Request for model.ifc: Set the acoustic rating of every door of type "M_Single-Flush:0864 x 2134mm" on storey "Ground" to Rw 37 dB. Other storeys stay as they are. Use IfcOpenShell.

First a look at what the model holds.

```python
import ifcopenshell
import ifcopenshell.util.element

model = ifcopenshell.open("model.ifc")
print(model.schema)
storey = next(s for s in model.by_type("IfcBuildingStorey") if s.Name == "Ground")
doors = [e for e in ifcopenshell.util.element.get_decomposition(storey) if e.is_a("IfcDoor")]
seen = {}
for e in doors:
    element_type = ifcopenshell.util.element.get_type(e)
    key = (element_type.Name if element_type != e and element_type else None, ifcopenshell.util.element.get_pset(e, "Pset_DoorCommon", "AcousticRating"))
    seen[key] = seen.get(key, 0) + 1
for (name, value), count in sorted(seen.items(), key=str):
    print(count, "x", name, "|", value)
```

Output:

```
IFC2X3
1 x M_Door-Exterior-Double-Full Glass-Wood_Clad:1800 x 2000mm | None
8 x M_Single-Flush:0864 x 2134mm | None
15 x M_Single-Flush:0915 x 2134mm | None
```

```python
import ifcopenshell
import ifcopenshell.api.pset
import ifcopenshell.util.element

model = ifcopenshell.open("model.ifc")

storey = next(s for s in model.by_type("IfcBuildingStorey") if s.Name == "Ground")
doors = [e for e in ifcopenshell.util.element.get_decomposition(storey) if e.is_a("IfcDoor")]

count = 0
for e in doors:
    element_type = ifcopenshell.util.element.get_type(e)
    if element_type in (None, e) or element_type.Name != "M_Single-Flush:0864 x 2134mm":
        continue
    # add_pset returns the element's existing set when there is one.
    pset = ifcopenshell.api.pset.add_pset(model, product=e, name="Pset_DoorCommon")
    ifcopenshell.api.pset.edit_pset(model, pset=pset, properties={"AcousticRating": "Rw 37 dB"})
    count += 1

print(count, "doors updated")

model.write("model_updated.ifc")
```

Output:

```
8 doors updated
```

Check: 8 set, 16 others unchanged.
